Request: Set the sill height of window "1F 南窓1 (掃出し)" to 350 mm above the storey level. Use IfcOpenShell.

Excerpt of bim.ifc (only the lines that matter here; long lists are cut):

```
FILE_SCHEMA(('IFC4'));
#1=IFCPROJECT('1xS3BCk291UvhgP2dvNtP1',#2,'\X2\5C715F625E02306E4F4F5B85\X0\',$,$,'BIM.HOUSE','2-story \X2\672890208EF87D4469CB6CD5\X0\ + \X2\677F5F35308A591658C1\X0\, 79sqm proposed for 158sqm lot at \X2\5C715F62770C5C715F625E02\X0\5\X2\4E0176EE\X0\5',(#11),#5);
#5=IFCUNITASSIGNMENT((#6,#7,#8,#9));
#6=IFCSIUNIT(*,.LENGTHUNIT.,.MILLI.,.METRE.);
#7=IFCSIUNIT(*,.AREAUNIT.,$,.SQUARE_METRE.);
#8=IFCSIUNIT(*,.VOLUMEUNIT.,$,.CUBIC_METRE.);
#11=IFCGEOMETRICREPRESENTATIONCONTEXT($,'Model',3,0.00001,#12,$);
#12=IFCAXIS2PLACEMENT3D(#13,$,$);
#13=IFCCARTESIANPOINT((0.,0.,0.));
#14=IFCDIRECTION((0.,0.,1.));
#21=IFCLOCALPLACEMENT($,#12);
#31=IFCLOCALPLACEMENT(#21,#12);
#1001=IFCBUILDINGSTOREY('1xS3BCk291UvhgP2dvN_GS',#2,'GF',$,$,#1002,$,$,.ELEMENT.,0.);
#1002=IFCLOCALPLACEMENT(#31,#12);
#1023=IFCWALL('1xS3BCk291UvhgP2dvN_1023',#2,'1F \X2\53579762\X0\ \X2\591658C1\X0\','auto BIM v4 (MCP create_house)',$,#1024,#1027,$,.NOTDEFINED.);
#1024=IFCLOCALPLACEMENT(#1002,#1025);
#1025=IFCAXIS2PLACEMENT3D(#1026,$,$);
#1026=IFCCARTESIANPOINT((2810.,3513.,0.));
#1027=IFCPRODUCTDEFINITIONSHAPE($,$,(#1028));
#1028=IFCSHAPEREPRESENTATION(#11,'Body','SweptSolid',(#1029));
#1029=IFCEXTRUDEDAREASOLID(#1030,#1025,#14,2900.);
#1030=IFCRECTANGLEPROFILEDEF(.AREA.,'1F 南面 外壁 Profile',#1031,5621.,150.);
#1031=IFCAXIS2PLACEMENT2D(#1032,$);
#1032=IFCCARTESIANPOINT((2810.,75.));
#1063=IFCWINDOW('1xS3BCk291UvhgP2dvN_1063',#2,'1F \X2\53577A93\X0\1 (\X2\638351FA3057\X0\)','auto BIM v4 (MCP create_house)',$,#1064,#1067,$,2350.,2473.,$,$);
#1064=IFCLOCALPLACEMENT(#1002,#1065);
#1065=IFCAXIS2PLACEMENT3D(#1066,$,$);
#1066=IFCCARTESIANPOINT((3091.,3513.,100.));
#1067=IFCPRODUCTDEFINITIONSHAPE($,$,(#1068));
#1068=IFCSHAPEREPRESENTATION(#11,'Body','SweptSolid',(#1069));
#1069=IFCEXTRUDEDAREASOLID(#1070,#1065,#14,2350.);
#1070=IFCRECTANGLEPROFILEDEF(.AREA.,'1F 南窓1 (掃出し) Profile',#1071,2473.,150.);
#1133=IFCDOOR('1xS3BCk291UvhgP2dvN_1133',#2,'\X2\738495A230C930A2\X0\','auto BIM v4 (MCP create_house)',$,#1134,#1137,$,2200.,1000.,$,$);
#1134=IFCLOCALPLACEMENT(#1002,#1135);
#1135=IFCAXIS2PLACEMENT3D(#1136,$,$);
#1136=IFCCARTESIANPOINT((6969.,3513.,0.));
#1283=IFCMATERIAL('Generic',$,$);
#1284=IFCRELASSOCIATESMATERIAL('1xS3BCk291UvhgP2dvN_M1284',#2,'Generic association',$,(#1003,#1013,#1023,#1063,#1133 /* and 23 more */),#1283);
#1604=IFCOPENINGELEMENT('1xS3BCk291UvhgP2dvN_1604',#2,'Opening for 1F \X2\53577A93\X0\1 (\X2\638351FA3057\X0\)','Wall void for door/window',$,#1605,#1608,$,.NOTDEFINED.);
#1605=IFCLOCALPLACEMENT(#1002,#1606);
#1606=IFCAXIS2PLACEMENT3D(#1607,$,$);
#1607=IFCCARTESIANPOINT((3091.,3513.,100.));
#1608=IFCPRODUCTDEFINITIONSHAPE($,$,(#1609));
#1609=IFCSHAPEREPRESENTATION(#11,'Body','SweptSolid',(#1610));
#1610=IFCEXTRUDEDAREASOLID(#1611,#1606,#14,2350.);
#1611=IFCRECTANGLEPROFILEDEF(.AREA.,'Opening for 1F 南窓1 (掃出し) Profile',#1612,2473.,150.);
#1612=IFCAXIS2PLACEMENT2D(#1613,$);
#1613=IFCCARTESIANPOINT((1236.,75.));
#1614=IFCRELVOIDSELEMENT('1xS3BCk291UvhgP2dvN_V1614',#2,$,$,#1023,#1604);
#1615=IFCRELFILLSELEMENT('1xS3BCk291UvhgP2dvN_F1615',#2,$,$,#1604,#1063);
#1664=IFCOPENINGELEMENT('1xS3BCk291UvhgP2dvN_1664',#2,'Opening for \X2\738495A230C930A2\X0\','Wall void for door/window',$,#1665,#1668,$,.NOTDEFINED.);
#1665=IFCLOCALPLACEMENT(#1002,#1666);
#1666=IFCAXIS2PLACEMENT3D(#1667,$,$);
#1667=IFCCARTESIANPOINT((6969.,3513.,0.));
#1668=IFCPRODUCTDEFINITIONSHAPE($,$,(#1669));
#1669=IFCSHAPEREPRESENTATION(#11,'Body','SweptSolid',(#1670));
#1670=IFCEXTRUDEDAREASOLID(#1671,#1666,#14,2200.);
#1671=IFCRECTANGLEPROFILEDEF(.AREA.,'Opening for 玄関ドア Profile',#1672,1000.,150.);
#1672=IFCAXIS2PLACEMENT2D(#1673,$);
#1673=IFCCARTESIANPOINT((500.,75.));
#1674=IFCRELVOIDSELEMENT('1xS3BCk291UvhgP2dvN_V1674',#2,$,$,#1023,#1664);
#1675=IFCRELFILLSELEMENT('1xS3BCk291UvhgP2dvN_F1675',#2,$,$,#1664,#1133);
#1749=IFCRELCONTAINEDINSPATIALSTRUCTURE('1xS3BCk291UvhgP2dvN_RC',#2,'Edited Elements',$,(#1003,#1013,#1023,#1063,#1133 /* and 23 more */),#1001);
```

```python
import numpy as np
import ifcopenshell
import ifcopenshell.api.geometry
import ifcopenshell.geom
import ifcopenshell.util.element
import ifcopenshell.util.placement
import ifcopenshell.util.shape
import ifcopenshell.util.unit

model = ifcopenshell.open("bim.ifc")
unit_scale = ifcopenshell.util.unit.calculate_unit_scale(model)

window = model.by_guid("1xS3BCk291UvhgP2dvN_1063")
opening = window.FillsVoids[0].RelatingOpeningElement
storey = ifcopenshell.util.element.get_container(window, ifc_class="IfcBuildingStorey")
level = ifcopenshell.util.placement.get_local_placement(storey.ObjectPlacement)[2, 3]

# The opening's origin need not be at the sill, so measure its lowest point.
shape = ifcopenshell.geom.create_shape(ifcopenshell.geom.settings(), opening)
bottom = ifcopenshell.util.shape.get_shape_bottom_elevation(shape, shape.geometry) / unit_scale
dz = level + 0.35 / unit_scale - bottom

shift = np.array([0.0, 0.0, dz])
# The window is not placed relative to its opening, so move both.
for product in (opening, window):
    matrix = ifcopenshell.util.placement.get_local_placement(product.ObjectPlacement)
    matrix[:3, 3] += shift
    ifcopenshell.api.geometry.edit_object_placement(model, product=product, matrix=matrix, is_si=False)

print(f"moved by {dz * unit_scale:+.3f} m")

model.write("bim-out.ifc")
```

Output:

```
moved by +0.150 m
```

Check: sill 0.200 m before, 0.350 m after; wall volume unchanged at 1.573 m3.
